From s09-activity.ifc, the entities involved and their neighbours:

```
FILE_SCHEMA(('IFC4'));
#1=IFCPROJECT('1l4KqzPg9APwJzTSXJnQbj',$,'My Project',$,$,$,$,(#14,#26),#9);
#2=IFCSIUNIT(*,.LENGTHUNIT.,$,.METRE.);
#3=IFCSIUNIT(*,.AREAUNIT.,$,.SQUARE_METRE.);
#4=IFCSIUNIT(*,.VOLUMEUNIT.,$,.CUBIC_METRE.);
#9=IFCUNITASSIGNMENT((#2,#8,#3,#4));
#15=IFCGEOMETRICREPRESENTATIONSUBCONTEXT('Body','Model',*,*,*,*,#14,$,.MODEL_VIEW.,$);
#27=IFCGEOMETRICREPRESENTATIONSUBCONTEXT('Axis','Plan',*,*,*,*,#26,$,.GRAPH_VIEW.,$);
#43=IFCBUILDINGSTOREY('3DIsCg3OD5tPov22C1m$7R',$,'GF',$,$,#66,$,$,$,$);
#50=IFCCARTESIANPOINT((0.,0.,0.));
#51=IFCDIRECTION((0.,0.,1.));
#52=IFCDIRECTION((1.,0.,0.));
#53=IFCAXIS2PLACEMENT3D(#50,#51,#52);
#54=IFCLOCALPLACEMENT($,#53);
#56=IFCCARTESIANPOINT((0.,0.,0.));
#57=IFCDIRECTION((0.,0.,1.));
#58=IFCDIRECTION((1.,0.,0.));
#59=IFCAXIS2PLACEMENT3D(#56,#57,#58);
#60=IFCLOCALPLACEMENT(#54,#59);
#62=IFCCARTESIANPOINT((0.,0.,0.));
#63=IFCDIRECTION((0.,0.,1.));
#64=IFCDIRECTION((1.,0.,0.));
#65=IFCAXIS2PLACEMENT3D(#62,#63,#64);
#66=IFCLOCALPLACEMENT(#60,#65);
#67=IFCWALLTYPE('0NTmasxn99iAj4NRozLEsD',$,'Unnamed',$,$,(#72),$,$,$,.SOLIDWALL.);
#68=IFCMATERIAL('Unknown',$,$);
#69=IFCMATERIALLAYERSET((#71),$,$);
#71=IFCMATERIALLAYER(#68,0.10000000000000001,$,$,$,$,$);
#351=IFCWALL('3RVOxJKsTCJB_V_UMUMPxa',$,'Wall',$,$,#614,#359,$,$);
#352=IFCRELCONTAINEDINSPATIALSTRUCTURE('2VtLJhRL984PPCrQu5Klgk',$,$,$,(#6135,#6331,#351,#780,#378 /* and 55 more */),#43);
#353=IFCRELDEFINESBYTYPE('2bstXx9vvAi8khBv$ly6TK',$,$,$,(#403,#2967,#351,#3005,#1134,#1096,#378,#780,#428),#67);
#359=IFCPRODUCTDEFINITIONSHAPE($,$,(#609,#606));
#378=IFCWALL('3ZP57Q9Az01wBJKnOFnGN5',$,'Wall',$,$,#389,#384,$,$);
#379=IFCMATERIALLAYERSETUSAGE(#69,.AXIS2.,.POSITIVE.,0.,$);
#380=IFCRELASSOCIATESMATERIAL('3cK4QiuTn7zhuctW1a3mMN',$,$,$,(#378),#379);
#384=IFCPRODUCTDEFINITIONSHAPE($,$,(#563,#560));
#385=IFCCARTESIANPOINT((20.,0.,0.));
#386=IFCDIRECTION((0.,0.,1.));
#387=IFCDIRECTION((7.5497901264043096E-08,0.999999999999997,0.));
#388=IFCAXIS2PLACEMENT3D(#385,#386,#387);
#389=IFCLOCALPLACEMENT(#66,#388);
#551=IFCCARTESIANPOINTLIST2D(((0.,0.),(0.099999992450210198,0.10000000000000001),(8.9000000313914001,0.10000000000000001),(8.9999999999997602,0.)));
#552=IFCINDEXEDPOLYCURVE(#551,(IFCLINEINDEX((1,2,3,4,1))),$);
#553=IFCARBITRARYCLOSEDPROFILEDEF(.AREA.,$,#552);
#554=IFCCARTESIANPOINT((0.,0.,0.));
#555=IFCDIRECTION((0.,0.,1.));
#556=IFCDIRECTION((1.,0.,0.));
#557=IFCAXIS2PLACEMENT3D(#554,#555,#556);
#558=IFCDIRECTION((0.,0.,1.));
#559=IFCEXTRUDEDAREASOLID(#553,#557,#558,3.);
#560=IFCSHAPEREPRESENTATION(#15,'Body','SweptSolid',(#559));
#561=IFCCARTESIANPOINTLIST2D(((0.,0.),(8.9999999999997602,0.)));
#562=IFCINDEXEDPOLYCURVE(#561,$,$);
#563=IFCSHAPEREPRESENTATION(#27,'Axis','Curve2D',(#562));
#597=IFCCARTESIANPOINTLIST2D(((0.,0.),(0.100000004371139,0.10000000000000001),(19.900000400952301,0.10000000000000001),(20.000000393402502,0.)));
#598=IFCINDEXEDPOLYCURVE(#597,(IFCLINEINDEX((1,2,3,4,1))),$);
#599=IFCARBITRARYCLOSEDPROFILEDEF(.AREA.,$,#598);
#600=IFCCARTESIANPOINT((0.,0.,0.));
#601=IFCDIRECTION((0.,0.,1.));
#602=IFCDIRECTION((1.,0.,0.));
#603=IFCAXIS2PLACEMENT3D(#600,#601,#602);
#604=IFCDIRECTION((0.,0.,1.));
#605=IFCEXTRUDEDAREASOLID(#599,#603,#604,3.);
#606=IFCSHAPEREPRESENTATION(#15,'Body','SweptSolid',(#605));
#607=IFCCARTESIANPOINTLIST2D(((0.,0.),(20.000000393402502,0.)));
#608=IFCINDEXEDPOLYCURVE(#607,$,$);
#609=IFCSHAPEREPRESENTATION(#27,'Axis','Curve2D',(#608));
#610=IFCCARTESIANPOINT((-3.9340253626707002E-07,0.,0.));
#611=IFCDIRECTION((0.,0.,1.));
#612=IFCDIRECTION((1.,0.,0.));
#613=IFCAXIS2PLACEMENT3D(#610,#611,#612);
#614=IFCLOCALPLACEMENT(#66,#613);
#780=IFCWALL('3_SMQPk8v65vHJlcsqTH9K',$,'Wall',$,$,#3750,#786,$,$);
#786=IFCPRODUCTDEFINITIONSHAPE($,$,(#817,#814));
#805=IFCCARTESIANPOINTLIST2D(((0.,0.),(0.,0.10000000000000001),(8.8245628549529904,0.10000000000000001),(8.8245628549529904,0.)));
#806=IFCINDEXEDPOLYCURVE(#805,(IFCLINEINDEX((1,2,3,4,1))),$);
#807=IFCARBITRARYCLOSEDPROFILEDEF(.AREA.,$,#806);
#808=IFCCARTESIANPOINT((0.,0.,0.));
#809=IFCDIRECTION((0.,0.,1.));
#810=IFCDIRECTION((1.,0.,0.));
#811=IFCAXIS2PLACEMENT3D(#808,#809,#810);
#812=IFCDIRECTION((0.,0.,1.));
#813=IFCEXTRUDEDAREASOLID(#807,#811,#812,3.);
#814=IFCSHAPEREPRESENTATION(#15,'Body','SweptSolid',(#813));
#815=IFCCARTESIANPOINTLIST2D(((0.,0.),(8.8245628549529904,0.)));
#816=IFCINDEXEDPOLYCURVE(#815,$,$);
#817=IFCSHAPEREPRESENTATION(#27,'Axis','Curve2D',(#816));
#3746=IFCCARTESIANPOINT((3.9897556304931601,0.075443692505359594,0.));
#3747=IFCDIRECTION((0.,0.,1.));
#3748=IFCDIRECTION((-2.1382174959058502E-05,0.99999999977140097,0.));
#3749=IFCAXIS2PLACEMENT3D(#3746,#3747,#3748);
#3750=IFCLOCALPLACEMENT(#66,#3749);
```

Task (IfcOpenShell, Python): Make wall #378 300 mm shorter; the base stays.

```python
import ifcopenshell
import ifcopenshell.geom
import ifcopenshell.util.representation
import ifcopenshell.util.shape
import ifcopenshell.util.unit

model = ifcopenshell.open("s09-activity.ifc")
unit_scale = ifcopenshell.util.unit.calculate_unit_scale(model)
settings = ifcopenshell.geom.settings()


def volume(element):
    """Net volume in cubic metres, openings subtracted."""
    shape = ifcopenshell.geom.create_shape(settings, element)
    return ifcopenshell.util.shape.get_volume(shape.geometry)


wall = model.by_id(378)
before = volume(wall)

body = ifcopenshell.util.representation.get_representation(wall, "Model", "Body")
solid = body.Items[0]
old_height = solid.Depth
solid.Depth -= 0.3 / unit_scale
after = volume(wall)

print(f"height {old_height:g} -> {solid.Depth:g}, volume {before:.3f} -> {after:.3f} m3")

model.write("s09-activity-out.ifc")
```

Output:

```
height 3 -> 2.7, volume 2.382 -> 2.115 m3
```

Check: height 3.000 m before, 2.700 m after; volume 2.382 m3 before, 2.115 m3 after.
